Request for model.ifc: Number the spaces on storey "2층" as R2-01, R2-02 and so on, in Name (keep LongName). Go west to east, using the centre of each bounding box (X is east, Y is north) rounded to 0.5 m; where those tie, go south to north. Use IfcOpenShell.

First a look at what the model holds.

```python
import ifcopenshell
import ifcopenshell.util.element
import ifcopenshell.util.placement

model = ifcopenshell.open("model.ifc")
print(model.schema)
storey = next(s for s in model.by_type("IfcBuildingStorey") if s.Name == "2층")
spaces = [e for e in ifcopenshell.util.element.get_decomposition(storey) if e.is_a("IfcSpace")]
for e in sorted(spaces, key=lambda e: e.id()):
    origin = ifcopenshell.util.placement.get_local_placement(e.ObjectPlacement)[:3, 3]
    print(e.id(), e.Name, e.LongName, origin.round(2) + 0.0, sep=" | ")
```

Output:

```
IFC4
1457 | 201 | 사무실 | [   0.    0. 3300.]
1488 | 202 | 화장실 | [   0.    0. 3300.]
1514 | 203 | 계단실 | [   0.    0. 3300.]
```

```python
import ifcopenshell
import ifcopenshell.geom
import ifcopenshell.util.element
import ifcopenshell.util.shape

model = ifcopenshell.open("model.ifc")
settings = ifcopenshell.geom.settings()
settings.set("use-world-coords", True)


def centre(element):
    shape = ifcopenshell.geom.create_shape(settings, element)
    return ifcopenshell.util.shape.get_bbox_centroid(shape.geometry)


storey = next(s for s in model.by_type("IfcBuildingStorey") if s.Name == "2층")
spaces = [e for e in ifcopenshell.util.element.get_decomposition(storey) if e.is_a("IfcSpace")]

# Insertion points can sit at a corner or the storey origin, so sort by the geometry (in metres).
centres = {e: centre(e) for e in spaces}
spaces.sort(key=lambda e: (round(centres[e][0] / 0.5), centres[e][1]))

for i, e in enumerate(spaces, start=1):
    number = f"R2-{i:02d}"
    e.Name = number
    print(e.id(), number)

model.write("model_rev.ifc")
```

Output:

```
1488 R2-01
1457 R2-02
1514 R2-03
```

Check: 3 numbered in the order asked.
